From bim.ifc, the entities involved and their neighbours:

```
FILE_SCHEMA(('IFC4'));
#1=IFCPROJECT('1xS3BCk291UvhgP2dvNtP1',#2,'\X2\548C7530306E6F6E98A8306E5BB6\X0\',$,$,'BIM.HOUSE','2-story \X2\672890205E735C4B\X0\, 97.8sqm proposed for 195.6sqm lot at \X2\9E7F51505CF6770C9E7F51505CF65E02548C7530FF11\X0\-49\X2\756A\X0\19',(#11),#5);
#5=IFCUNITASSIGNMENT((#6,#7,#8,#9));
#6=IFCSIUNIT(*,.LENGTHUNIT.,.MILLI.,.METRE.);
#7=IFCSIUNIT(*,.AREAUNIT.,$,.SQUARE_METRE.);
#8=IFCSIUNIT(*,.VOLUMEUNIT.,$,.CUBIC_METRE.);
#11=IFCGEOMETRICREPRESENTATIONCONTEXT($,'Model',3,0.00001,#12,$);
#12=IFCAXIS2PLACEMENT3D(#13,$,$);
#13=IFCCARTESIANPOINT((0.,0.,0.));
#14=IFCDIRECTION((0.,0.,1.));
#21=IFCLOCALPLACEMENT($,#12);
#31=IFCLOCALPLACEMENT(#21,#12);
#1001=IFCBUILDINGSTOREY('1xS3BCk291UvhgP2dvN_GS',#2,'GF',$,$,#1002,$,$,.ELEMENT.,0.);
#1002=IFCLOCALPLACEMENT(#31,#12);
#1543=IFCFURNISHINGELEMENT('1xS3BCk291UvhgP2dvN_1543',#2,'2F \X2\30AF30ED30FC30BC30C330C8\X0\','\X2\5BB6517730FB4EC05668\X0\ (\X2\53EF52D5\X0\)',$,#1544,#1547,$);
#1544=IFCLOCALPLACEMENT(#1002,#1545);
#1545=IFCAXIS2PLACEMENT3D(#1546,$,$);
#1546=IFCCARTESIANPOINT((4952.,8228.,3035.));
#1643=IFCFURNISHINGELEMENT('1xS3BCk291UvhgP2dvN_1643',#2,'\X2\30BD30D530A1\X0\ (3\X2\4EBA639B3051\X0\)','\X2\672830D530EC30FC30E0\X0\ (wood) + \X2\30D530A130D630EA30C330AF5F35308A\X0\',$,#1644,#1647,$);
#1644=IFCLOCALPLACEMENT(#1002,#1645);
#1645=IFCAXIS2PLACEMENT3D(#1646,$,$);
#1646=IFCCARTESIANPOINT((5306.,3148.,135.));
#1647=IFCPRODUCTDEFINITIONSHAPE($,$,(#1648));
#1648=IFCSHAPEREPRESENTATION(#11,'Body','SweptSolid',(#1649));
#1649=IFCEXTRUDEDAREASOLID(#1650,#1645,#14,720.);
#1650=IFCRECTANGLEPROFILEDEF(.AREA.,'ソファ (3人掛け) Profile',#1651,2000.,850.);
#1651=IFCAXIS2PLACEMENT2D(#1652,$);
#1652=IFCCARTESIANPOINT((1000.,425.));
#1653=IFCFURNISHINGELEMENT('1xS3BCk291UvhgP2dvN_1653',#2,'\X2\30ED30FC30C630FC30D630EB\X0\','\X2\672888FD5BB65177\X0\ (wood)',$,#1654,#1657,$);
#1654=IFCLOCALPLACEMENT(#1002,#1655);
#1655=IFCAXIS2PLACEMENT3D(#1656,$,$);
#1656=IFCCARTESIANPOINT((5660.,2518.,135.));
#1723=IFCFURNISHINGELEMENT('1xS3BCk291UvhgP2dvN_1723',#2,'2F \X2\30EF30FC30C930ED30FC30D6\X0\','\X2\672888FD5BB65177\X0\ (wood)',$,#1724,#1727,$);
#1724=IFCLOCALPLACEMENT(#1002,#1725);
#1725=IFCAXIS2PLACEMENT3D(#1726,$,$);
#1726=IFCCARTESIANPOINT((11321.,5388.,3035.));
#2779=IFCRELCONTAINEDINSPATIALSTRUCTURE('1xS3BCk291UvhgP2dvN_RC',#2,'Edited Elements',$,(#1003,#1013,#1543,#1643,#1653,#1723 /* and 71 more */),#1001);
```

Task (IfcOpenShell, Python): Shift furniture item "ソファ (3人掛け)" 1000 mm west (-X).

```python
import ifcopenshell
import ifcopenshell.api.geometry
import ifcopenshell.util.placement
import ifcopenshell.util.unit

model = ifcopenshell.open("bim.ifc")
unit_scale = ifcopenshell.util.unit.calculate_unit_scale(model)

item = model.by_id(1643)
matrix = ifcopenshell.util.placement.get_local_placement(item.ObjectPlacement)
matrix[0, 3] -= 1 / unit_scale
ifcopenshell.api.geometry.edit_object_placement(model, product=item, matrix=matrix, is_si=False)

print(ifcopenshell.util.placement.get_local_placement(item.ObjectPlacement).round(3) + 0.0)

model.write("bim_edited.ifc")
```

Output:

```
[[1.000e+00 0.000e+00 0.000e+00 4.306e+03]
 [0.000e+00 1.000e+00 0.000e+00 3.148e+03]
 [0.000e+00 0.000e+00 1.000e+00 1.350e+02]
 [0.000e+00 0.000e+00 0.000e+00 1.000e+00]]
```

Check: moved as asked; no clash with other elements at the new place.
